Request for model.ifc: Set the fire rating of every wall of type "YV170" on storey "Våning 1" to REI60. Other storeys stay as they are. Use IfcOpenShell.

First a look at what the model holds.

```python
import ifcopenshell
import ifcopenshell.util.element

model = ifcopenshell.open("model.ifc")
print(model.schema)
storey = next(s for s in model.by_type("IfcBuildingStorey") if s.Name == "Våning 1")
walls = [e for e in ifcopenshell.util.element.get_decomposition(storey) if e.is_a("IfcWall")]
seen = {}
for e in walls:
    element_type = ifcopenshell.util.element.get_type(e)
    key = (element_type.Name if element_type != e and element_type else None, ifcopenshell.util.element.get_pset(e, "Pset_WallCommon", "FireRating"))
    seen[key] = seen.get(key, 0) + 1
for (name, value), count in sorted(seen.items(), key=str):
    print(count, "x", name, "|", value)
```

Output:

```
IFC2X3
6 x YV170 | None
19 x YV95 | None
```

```python
import ifcopenshell
import ifcopenshell.api.pset
import ifcopenshell.util.element

model = ifcopenshell.open("model.ifc")

storey = next(s for s in model.by_type("IfcBuildingStorey") if s.Name == "Våning 1")
walls = [e for e in ifcopenshell.util.element.get_decomposition(storey) if e.is_a("IfcWall")]

count = 0
for e in walls:
    element_type = ifcopenshell.util.element.get_type(e)
    if element_type in (None, e) or element_type.Name != "YV170":
        continue
    # add_pset returns the element's existing set when there is one.
    pset = ifcopenshell.api.pset.add_pset(model, product=e, name="Pset_WallCommon")
    ifcopenshell.api.pset.edit_pset(model, pset=pset, properties={"FireRating": "REI60"})
    count += 1

print(count, "walls updated")

model.write("model-out.ifc")
```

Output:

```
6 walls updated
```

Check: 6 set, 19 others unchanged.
